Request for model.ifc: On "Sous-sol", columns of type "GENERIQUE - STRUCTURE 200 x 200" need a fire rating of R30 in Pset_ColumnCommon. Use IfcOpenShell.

First a look at what the model holds.

```python
import ifcopenshell
import ifcopenshell.util.element

model = ifcopenshell.open("model.ifc")
print(model.schema)
storey = next(s for s in model.by_type("IfcBuildingStorey") if s.Name == "Sous-sol")
columns = [e for e in ifcopenshell.util.element.get_decomposition(storey) if e.is_a("IfcColumn")]
seen = {}
for e in columns:
    element_type = ifcopenshell.util.element.get_type(e)
    key = (element_type.Name if element_type != e and element_type else None, ifcopenshell.util.element.get_pset(e, "Pset_ColumnCommon", "FireRating"))
    seen[key] = seen.get(key, 0) + 1
for (name, value), count in sorted(seen.items(), key=str):
    print(count, "x", name, "|", value)
```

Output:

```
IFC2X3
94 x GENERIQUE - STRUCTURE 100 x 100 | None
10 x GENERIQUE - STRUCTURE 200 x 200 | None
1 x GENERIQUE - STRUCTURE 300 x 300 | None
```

```python
import ifcopenshell
import ifcopenshell.api.pset
import ifcopenshell.util.element

model = ifcopenshell.open("model.ifc")

storey = next(s for s in model.by_type("IfcBuildingStorey") if s.Name == "Sous-sol")
columns = [e for e in ifcopenshell.util.element.get_decomposition(storey) if e.is_a("IfcColumn")]

count = 0
for e in columns:
    element_type = ifcopenshell.util.element.get_type(e)
    if element_type in (None, e) or element_type.Name != "GENERIQUE - STRUCTURE 200 x 200":
        continue
    # add_pset returns the element's existing set when there is one.
    pset = ifcopenshell.api.pset.add_pset(model, product=e, name="Pset_ColumnCommon")
    ifcopenshell.api.pset.edit_pset(model, pset=pset, properties={"FireRating": "R30"})
    count += 1

print(count, "columns updated")

model.write("model_updated.ifc")
```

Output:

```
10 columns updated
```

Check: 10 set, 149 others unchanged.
